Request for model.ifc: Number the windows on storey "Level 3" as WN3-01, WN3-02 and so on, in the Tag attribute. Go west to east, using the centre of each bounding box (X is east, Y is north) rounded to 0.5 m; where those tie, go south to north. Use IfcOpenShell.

First a look at what the model holds.

```python
import ifcopenshell
import ifcopenshell.util.element
import ifcopenshell.util.placement

model = ifcopenshell.open("model.ifc")
print(model.schema)
storey = next(s for s in model.by_type("IfcBuildingStorey") if s.Name == "Level 3")
windows = [e for e in ifcopenshell.util.element.get_decomposition(storey) if e.is_a("IfcWindow")]
for e in sorted(windows, key=lambda e: e.id()):
    origin = ifcopenshell.util.placement.get_local_placement(e.ObjectPlacement)[:3, 3]
    print(e.id(), e.Tag, e.Name, origin.round(2) + 0.0, sep=" | ")
```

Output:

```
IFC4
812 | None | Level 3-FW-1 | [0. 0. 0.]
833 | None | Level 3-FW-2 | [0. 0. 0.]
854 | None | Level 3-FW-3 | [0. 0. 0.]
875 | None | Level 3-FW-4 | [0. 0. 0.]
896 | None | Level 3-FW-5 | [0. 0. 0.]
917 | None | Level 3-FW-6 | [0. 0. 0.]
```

```python
import ifcopenshell
import ifcopenshell.geom
import ifcopenshell.util.element
import ifcopenshell.util.shape

model = ifcopenshell.open("model.ifc")
settings = ifcopenshell.geom.settings()
settings.set("use-world-coords", True)


def centre(element):
    shape = ifcopenshell.geom.create_shape(settings, element)
    return ifcopenshell.util.shape.get_bbox_centroid(shape.geometry)


storey = next(s for s in model.by_type("IfcBuildingStorey") if s.Name == "Level 3")
windows = [e for e in ifcopenshell.util.element.get_decomposition(storey) if e.is_a("IfcWindow")]

# Insertion points can sit at a corner or the storey origin, so sort by the geometry (in metres).
centres = {e: centre(e) for e in windows}
windows.sort(key=lambda e: (round(centres[e][0] / 0.5), centres[e][1]))

for i, e in enumerate(windows, start=1):
    number = f"WN3-{i:02d}"
    e.Tag = number
    print(e.id(), number)

model.write("model_rev.ifc")
```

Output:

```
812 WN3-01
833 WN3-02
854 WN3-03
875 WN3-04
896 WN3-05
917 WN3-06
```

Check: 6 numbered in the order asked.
